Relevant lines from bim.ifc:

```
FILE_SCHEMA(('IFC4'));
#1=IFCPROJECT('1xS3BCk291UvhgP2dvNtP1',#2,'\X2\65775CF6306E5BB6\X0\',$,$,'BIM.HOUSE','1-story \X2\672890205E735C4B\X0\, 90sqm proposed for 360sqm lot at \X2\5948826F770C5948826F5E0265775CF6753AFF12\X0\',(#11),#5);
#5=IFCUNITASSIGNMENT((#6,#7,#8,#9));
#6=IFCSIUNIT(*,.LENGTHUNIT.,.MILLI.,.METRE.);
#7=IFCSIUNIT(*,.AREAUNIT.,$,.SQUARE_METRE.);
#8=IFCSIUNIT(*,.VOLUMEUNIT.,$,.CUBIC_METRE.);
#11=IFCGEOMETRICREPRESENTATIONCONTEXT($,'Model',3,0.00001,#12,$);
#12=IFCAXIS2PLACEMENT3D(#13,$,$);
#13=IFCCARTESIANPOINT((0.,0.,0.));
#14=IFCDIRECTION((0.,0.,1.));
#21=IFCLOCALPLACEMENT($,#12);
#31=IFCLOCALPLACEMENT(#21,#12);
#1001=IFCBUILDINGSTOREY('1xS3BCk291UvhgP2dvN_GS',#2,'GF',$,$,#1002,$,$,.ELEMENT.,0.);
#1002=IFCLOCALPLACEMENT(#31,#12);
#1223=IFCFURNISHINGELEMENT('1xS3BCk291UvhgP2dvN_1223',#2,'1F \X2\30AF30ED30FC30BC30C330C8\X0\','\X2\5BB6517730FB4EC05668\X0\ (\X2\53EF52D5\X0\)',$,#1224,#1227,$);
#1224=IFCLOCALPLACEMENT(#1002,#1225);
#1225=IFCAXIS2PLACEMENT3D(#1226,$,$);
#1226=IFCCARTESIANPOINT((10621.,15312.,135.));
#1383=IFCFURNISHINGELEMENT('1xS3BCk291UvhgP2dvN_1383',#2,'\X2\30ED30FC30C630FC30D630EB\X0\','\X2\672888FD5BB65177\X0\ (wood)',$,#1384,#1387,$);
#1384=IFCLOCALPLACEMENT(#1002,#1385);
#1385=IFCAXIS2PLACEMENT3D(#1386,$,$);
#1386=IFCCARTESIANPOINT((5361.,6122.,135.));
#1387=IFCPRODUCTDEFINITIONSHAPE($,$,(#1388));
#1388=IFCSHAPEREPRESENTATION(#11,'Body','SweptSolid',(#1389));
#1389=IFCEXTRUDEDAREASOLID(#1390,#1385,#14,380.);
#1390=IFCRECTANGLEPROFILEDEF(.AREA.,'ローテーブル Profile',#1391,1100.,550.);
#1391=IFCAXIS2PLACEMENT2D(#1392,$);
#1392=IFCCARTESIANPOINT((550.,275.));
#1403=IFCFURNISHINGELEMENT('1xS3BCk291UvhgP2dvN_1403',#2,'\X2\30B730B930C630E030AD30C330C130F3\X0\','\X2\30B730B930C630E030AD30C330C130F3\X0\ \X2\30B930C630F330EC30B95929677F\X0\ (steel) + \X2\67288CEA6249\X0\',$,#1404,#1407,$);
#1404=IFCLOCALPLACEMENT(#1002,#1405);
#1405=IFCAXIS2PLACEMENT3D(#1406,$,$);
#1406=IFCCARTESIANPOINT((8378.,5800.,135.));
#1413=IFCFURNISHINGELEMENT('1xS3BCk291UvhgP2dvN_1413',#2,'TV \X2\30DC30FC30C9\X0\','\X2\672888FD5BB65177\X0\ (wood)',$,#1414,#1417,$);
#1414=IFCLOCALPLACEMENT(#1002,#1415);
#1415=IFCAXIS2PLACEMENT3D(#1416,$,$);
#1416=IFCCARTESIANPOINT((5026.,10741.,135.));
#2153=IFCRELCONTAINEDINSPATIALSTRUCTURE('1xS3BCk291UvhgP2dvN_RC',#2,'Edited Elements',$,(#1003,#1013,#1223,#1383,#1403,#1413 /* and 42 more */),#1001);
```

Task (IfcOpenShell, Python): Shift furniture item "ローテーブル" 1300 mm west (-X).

```python
import ifcopenshell
import ifcopenshell.api.geometry
import ifcopenshell.util.placement

model = ifcopenshell.open("bim.ifc")

item = model.by_guid("1xS3BCk291UvhgP2dvN_1383")
matrix = ifcopenshell.util.placement.get_local_placement(item.ObjectPlacement)
matrix[0, 3] -= 1300.0
ifcopenshell.api.geometry.edit_object_placement(model, product=item, matrix=matrix, is_si=False)

print(ifcopenshell.util.placement.get_local_placement(item.ObjectPlacement).round(3) + 0.0)

model.write("bim_edited.ifc")
```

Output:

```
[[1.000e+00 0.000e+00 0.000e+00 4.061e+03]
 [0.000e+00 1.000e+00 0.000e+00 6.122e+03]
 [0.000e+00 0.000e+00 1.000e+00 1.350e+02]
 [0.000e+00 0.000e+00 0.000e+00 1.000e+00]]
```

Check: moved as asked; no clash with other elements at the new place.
